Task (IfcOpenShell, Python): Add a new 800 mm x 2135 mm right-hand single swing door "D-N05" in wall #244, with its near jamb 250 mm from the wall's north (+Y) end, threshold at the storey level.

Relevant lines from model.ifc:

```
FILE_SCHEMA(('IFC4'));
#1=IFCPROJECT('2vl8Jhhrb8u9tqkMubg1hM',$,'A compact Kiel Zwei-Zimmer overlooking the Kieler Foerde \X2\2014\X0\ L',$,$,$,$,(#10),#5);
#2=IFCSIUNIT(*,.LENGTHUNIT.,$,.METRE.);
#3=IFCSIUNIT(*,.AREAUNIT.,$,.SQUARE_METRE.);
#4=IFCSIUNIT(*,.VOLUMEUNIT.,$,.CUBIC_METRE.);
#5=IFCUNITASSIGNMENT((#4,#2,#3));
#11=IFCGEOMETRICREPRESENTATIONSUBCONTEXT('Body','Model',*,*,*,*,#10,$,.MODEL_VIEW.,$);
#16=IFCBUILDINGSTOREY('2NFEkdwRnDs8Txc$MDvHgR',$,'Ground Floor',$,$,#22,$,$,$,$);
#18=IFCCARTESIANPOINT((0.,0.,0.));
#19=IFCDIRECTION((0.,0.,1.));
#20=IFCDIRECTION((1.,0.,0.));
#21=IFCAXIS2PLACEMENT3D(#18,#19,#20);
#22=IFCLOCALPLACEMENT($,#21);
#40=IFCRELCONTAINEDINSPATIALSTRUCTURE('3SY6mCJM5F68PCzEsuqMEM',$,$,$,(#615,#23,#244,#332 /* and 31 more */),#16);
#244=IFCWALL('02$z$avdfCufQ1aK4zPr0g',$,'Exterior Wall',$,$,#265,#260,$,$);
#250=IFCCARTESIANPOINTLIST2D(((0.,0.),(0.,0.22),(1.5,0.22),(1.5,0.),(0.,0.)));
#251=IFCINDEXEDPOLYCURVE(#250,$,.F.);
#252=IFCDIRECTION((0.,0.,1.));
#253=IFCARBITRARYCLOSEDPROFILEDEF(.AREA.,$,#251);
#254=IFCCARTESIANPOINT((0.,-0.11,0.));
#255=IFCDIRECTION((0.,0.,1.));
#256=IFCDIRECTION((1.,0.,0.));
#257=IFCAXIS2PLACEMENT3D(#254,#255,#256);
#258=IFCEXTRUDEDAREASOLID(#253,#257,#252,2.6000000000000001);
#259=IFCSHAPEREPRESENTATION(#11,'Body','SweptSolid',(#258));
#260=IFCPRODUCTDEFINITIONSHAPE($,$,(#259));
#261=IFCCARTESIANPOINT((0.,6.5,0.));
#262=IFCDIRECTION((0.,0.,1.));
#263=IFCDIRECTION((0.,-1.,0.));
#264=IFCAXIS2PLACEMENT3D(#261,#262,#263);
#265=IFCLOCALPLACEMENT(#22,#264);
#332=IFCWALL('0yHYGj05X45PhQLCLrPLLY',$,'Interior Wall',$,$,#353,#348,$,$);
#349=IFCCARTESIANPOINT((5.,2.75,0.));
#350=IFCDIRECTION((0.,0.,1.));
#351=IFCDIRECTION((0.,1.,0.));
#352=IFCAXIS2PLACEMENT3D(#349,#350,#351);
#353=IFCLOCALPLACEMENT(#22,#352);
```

```python
import numpy as np
import ifcopenshell
import ifcopenshell.api.feature
import ifcopenshell.api.geometry
import ifcopenshell.api.root
import ifcopenshell.api.spatial
import ifcopenshell.geom
import ifcopenshell.util.element
import ifcopenshell.util.placement
import ifcopenshell.util.representation
import ifcopenshell.util.shape
import ifcopenshell.util.unit

model = ifcopenshell.open("model.ifc")
unit_scale = ifcopenshell.util.unit.calculate_unit_scale(model)
settings = ifcopenshell.geom.settings()


def volume(element):
    """Net volume in cubic metres, openings subtracted."""
    shape = ifcopenshell.geom.create_shape(settings, element)
    return ifcopenshell.util.shape.get_volume(shape.geometry)


wall = model.by_id(244)
storey = ifcopenshell.util.element.get_container(wall, ifc_class="IfcBuildingStorey")
context = ifcopenshell.util.representation.get_context(model, "Model", "Body", "MODEL_VIEW")
before = volume(wall)

width, height, from_end, sill = 0.8, 2.135, 0.25, 0.0  # metres

# The wall runs along its own X axis, and the end named is its -X end.
wall_shape = ifcopenshell.geom.create_shape(settings, wall)
x, y, z = ifcopenshell.util.shape.get_vertices(wall_shape.geometry).T
start = x.min() + from_end
face, thickness = float(y.min()), float(y.max() - y.min())
wall_matrix = ifcopenshell.util.placement.get_local_placement(wall.ObjectPlacement)
level = ifcopenshell.util.placement.get_local_placement(storey.ObjectPlacement)[2, 3]


def in_wall(x, y):
    """Placement at x, y metres in the wall's axes, at sill height."""
    matrix = wall_matrix.copy()
    matrix[:, 3] = wall_matrix @ np.array([x / unit_scale, y / unit_scale, 0.0, 1.0])
    matrix[2, 3] = level + sill / unit_scale
    return matrix


# Opening: a box that overshoots both wall faces by 50 mm.
opening = ifcopenshell.api.root.create_entity(model, ifc_class="IfcOpeningElement", predefined_type="OPENING")
box = ifcopenshell.api.geometry.add_wall_representation(
    model, context=context, length=width, height=height, thickness=thickness + 0.1
)
ifcopenshell.api.geometry.assign_representation(model, product=opening, representation=box)
ifcopenshell.api.geometry.edit_object_placement(model, product=opening, matrix=in_wall(start, face - 0.05), is_si=False)
ifcopenshell.api.feature.add_feature(model, feature=opening, element=wall)

door = ifcopenshell.api.root.create_entity(model, ifc_class="IfcDoor", name="D-N05", predefined_type="DOOR")
door.OverallWidth, door.OverallHeight = width / unit_scale, height / unit_scale
door.OperationType = "SINGLE_SWING_RIGHT"
body = ifcopenshell.api.geometry.add_door_representation(
    model,
    context=context,
    overall_width=door.OverallWidth,
    overall_height=door.OverallHeight,
    operation_type="SINGLE_SWING_RIGHT",
    lining_properties={"LiningDepth": thickness / unit_scale, "ThresholdDepth": thickness / unit_scale},
)
ifcopenshell.api.geometry.assign_representation(model, product=door, representation=body)
ifcopenshell.api.spatial.assign_container(model, products=[door], relating_structure=storey)
ifcopenshell.api.feature.add_filling(model, opening=opening, element=door)

# The lining spans the wall, so the door starts at the wall face.
ifcopenshell.api.geometry.edit_object_placement(model, product=door, matrix=in_wall(start, face), is_si=False)

after = volume(wall)

print(f"wall volume {before:.3f} -> {after:.3f} m3")

model.write("model_rev.ifc")
```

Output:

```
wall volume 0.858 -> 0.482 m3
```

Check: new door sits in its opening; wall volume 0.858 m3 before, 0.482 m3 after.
